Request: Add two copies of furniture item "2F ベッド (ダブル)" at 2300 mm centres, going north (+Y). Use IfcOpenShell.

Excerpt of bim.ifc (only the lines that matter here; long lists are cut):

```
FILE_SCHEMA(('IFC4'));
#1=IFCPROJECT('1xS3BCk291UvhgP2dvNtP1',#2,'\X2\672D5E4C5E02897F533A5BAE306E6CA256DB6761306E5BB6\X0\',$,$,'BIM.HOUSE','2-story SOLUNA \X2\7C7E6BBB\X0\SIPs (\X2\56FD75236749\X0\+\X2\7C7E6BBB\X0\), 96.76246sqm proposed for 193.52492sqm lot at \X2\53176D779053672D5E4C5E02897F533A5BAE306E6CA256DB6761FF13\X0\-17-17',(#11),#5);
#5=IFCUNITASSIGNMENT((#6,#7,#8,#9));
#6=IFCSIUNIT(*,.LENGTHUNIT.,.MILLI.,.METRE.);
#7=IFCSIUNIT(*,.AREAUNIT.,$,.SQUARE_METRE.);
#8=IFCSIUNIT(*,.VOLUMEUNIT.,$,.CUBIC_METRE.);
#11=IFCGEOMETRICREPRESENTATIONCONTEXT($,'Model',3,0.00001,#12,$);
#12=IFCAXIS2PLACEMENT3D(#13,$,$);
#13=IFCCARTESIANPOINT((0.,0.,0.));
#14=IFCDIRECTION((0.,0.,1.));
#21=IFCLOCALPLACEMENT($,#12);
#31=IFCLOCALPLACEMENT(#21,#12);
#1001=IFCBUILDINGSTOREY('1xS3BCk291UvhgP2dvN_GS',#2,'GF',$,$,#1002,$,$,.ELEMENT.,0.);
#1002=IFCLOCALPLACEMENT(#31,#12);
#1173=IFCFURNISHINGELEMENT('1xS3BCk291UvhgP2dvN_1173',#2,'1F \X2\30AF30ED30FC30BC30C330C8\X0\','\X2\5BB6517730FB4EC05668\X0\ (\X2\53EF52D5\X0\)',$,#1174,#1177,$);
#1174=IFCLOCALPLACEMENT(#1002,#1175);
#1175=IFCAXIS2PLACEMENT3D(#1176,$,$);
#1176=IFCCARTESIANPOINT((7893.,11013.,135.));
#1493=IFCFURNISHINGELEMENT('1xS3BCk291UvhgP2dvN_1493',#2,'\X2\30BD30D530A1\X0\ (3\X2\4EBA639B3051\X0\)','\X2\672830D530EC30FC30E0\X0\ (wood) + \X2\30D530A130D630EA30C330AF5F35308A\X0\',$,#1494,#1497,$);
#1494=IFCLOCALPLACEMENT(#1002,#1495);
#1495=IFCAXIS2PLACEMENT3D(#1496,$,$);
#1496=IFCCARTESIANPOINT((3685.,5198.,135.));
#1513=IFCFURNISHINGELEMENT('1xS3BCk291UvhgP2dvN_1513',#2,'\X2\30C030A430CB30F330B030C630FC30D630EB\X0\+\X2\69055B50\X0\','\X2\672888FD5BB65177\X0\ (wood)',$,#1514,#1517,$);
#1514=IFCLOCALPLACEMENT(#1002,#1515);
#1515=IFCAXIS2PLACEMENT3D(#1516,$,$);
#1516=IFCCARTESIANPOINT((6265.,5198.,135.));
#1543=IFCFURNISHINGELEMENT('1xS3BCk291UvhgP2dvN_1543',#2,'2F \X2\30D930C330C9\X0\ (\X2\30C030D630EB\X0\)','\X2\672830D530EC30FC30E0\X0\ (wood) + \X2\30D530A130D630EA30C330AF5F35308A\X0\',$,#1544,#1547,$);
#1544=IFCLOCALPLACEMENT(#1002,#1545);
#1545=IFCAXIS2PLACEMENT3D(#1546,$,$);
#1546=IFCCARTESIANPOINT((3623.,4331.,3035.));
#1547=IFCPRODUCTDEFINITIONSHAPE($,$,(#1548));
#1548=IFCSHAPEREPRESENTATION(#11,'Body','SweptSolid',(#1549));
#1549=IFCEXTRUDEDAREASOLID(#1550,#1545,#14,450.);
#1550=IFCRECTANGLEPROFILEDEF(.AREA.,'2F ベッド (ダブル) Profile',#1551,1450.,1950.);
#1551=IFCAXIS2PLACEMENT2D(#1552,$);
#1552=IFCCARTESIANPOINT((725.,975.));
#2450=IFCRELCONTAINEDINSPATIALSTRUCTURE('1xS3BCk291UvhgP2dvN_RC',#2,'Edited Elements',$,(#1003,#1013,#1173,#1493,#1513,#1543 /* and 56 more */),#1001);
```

```python
import numpy as np
import ifcopenshell
import ifcopenshell.api.geometry
import ifcopenshell.api.root
import ifcopenshell.util.element
import ifcopenshell.util.placement
import ifcopenshell.util.unit

model = ifcopenshell.open("bim.ifc")
unit_scale = ifcopenshell.util.unit.calculate_unit_scale(model)


def reuse_history(source, copy):
    """copy_class also copies each property set's owner history, people and application; keep the originals."""
    for rel in copy.IsDefinedBy:
        if rel.is_a("IfcRelDefinesByProperties") and (history := rel.RelatingPropertyDefinition.OwnerHistory):
            rel.RelatingPropertyDefinition.OwnerHistory = source.OwnerHistory
            ifcopenshell.util.element.remove_deep2(model, history)


source = model.by_guid("1xS3BCk291UvhgP2dvN_1543")
base = ifcopenshell.util.placement.get_local_placement(source.ObjectPlacement)
step = np.array([0.0, 1.0, 0.0]) * 2.3 / unit_scale

for i in range(1, 3):
    copy = ifcopenshell.api.root.copy_class(model, product=source)
    copy.Representation = ifcopenshell.util.element.copy_deep(
        model, source.Representation, exclude=["IfcGeometricRepresentationContext", "IfcRepresentationMap"]
    )
    reuse_history(source, copy)
    matrix = base.copy()
    matrix[:3, 3] += i * step
    print("added at", matrix[:3, 3].round(3) + 0.0)
    ifcopenshell.api.geometry.edit_object_placement(model, product=copy, matrix=matrix, is_si=False)

model.write("bim_edited.ifc")
```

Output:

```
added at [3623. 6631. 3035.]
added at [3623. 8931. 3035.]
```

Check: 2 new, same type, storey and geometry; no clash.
